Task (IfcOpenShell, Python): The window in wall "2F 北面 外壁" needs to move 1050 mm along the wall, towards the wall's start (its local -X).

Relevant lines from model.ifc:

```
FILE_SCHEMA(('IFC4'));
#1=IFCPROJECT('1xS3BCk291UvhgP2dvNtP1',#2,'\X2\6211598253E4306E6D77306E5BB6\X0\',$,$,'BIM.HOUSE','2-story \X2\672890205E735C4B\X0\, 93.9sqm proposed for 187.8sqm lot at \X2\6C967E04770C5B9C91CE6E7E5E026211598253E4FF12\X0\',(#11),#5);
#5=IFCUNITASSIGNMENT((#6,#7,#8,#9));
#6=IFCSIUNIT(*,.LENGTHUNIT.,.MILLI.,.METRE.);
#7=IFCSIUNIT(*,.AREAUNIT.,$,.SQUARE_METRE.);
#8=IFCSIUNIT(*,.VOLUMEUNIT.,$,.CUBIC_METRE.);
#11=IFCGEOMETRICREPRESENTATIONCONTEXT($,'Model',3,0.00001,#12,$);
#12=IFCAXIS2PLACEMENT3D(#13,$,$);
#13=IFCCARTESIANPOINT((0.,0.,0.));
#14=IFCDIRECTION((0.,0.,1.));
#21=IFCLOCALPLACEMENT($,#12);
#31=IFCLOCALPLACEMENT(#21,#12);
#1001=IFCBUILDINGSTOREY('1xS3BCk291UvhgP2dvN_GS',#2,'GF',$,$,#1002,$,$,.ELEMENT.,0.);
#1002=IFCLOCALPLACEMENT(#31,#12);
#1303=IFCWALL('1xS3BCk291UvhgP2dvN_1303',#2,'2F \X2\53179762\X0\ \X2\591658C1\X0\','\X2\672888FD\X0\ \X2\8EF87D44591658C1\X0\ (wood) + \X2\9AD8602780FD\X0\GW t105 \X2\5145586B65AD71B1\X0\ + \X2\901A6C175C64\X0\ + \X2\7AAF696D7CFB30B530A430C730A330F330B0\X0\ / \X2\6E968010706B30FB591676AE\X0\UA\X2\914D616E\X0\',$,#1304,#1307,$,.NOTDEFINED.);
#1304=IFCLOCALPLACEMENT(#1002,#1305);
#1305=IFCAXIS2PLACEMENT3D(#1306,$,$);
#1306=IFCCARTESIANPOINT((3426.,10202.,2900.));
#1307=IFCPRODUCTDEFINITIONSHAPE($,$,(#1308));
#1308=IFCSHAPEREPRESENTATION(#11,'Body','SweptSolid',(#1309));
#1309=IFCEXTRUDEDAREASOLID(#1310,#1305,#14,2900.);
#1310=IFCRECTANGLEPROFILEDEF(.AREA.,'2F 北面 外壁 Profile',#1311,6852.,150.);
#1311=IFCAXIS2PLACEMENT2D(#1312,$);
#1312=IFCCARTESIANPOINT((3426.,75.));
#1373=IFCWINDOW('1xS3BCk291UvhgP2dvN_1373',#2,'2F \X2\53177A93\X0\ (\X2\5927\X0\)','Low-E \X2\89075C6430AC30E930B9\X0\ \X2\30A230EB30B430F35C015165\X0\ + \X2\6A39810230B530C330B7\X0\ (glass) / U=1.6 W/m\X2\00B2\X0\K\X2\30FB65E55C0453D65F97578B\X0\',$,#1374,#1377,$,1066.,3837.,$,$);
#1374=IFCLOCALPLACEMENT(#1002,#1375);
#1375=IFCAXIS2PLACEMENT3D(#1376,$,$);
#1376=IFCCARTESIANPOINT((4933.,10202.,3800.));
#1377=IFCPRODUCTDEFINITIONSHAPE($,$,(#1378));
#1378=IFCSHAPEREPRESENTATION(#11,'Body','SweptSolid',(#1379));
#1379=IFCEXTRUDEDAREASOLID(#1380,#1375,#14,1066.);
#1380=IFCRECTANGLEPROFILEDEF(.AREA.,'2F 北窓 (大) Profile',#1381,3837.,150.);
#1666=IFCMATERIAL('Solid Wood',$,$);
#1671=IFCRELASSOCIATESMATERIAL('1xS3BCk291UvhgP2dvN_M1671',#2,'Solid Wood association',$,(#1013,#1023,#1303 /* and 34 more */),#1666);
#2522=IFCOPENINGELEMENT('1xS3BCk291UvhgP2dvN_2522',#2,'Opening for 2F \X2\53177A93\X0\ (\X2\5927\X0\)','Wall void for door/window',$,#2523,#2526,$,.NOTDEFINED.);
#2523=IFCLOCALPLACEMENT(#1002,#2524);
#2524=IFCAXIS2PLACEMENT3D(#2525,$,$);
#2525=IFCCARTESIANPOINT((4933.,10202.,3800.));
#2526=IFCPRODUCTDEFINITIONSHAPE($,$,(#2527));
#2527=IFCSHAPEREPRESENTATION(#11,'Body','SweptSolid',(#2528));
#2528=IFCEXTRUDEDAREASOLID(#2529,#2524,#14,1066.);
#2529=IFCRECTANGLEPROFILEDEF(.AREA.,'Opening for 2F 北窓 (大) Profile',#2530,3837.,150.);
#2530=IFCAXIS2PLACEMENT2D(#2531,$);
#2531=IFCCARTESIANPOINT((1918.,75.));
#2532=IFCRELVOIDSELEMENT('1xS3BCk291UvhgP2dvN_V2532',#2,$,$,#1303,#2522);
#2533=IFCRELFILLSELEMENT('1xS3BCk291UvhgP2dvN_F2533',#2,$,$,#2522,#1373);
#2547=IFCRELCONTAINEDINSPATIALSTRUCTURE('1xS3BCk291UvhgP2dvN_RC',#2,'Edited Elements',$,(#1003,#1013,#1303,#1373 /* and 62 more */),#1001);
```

```python
import ifcopenshell
import ifcopenshell.api.geometry
import ifcopenshell.util.placement
import ifcopenshell.util.unit

model = ifcopenshell.open("model.ifc")
unit_scale = ifcopenshell.util.unit.calculate_unit_scale(model)

window = model.by_guid("1xS3BCk291UvhgP2dvN_1373")
opening = window.FillsVoids[0].RelatingOpeningElement
wall = opening.VoidsElements[0].RelatingBuildingElement

wall_matrix = ifcopenshell.util.placement.get_local_placement(wall.ObjectPlacement)
shift = wall_matrix[:3, 0] * -1.05 / unit_scale
before = ifcopenshell.util.placement.get_local_placement(window.ObjectPlacement)[:3, 3].copy()

# The window is not placed relative to its opening, so move both.
for product in (opening, window):
    matrix = ifcopenshell.util.placement.get_local_placement(product.ObjectPlacement)
    matrix[:3, 3] += shift
    ifcopenshell.api.geometry.edit_object_placement(model, product=product, matrix=matrix, is_si=False)

after = ifcopenshell.util.placement.get_local_placement(window.ObjectPlacement)[:3, 3]
print("window moved by", (after - before).round(3) + 0.0)

model.write("model-out.ifc")
```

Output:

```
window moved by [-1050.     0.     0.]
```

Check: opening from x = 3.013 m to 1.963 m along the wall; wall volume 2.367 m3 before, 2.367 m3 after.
